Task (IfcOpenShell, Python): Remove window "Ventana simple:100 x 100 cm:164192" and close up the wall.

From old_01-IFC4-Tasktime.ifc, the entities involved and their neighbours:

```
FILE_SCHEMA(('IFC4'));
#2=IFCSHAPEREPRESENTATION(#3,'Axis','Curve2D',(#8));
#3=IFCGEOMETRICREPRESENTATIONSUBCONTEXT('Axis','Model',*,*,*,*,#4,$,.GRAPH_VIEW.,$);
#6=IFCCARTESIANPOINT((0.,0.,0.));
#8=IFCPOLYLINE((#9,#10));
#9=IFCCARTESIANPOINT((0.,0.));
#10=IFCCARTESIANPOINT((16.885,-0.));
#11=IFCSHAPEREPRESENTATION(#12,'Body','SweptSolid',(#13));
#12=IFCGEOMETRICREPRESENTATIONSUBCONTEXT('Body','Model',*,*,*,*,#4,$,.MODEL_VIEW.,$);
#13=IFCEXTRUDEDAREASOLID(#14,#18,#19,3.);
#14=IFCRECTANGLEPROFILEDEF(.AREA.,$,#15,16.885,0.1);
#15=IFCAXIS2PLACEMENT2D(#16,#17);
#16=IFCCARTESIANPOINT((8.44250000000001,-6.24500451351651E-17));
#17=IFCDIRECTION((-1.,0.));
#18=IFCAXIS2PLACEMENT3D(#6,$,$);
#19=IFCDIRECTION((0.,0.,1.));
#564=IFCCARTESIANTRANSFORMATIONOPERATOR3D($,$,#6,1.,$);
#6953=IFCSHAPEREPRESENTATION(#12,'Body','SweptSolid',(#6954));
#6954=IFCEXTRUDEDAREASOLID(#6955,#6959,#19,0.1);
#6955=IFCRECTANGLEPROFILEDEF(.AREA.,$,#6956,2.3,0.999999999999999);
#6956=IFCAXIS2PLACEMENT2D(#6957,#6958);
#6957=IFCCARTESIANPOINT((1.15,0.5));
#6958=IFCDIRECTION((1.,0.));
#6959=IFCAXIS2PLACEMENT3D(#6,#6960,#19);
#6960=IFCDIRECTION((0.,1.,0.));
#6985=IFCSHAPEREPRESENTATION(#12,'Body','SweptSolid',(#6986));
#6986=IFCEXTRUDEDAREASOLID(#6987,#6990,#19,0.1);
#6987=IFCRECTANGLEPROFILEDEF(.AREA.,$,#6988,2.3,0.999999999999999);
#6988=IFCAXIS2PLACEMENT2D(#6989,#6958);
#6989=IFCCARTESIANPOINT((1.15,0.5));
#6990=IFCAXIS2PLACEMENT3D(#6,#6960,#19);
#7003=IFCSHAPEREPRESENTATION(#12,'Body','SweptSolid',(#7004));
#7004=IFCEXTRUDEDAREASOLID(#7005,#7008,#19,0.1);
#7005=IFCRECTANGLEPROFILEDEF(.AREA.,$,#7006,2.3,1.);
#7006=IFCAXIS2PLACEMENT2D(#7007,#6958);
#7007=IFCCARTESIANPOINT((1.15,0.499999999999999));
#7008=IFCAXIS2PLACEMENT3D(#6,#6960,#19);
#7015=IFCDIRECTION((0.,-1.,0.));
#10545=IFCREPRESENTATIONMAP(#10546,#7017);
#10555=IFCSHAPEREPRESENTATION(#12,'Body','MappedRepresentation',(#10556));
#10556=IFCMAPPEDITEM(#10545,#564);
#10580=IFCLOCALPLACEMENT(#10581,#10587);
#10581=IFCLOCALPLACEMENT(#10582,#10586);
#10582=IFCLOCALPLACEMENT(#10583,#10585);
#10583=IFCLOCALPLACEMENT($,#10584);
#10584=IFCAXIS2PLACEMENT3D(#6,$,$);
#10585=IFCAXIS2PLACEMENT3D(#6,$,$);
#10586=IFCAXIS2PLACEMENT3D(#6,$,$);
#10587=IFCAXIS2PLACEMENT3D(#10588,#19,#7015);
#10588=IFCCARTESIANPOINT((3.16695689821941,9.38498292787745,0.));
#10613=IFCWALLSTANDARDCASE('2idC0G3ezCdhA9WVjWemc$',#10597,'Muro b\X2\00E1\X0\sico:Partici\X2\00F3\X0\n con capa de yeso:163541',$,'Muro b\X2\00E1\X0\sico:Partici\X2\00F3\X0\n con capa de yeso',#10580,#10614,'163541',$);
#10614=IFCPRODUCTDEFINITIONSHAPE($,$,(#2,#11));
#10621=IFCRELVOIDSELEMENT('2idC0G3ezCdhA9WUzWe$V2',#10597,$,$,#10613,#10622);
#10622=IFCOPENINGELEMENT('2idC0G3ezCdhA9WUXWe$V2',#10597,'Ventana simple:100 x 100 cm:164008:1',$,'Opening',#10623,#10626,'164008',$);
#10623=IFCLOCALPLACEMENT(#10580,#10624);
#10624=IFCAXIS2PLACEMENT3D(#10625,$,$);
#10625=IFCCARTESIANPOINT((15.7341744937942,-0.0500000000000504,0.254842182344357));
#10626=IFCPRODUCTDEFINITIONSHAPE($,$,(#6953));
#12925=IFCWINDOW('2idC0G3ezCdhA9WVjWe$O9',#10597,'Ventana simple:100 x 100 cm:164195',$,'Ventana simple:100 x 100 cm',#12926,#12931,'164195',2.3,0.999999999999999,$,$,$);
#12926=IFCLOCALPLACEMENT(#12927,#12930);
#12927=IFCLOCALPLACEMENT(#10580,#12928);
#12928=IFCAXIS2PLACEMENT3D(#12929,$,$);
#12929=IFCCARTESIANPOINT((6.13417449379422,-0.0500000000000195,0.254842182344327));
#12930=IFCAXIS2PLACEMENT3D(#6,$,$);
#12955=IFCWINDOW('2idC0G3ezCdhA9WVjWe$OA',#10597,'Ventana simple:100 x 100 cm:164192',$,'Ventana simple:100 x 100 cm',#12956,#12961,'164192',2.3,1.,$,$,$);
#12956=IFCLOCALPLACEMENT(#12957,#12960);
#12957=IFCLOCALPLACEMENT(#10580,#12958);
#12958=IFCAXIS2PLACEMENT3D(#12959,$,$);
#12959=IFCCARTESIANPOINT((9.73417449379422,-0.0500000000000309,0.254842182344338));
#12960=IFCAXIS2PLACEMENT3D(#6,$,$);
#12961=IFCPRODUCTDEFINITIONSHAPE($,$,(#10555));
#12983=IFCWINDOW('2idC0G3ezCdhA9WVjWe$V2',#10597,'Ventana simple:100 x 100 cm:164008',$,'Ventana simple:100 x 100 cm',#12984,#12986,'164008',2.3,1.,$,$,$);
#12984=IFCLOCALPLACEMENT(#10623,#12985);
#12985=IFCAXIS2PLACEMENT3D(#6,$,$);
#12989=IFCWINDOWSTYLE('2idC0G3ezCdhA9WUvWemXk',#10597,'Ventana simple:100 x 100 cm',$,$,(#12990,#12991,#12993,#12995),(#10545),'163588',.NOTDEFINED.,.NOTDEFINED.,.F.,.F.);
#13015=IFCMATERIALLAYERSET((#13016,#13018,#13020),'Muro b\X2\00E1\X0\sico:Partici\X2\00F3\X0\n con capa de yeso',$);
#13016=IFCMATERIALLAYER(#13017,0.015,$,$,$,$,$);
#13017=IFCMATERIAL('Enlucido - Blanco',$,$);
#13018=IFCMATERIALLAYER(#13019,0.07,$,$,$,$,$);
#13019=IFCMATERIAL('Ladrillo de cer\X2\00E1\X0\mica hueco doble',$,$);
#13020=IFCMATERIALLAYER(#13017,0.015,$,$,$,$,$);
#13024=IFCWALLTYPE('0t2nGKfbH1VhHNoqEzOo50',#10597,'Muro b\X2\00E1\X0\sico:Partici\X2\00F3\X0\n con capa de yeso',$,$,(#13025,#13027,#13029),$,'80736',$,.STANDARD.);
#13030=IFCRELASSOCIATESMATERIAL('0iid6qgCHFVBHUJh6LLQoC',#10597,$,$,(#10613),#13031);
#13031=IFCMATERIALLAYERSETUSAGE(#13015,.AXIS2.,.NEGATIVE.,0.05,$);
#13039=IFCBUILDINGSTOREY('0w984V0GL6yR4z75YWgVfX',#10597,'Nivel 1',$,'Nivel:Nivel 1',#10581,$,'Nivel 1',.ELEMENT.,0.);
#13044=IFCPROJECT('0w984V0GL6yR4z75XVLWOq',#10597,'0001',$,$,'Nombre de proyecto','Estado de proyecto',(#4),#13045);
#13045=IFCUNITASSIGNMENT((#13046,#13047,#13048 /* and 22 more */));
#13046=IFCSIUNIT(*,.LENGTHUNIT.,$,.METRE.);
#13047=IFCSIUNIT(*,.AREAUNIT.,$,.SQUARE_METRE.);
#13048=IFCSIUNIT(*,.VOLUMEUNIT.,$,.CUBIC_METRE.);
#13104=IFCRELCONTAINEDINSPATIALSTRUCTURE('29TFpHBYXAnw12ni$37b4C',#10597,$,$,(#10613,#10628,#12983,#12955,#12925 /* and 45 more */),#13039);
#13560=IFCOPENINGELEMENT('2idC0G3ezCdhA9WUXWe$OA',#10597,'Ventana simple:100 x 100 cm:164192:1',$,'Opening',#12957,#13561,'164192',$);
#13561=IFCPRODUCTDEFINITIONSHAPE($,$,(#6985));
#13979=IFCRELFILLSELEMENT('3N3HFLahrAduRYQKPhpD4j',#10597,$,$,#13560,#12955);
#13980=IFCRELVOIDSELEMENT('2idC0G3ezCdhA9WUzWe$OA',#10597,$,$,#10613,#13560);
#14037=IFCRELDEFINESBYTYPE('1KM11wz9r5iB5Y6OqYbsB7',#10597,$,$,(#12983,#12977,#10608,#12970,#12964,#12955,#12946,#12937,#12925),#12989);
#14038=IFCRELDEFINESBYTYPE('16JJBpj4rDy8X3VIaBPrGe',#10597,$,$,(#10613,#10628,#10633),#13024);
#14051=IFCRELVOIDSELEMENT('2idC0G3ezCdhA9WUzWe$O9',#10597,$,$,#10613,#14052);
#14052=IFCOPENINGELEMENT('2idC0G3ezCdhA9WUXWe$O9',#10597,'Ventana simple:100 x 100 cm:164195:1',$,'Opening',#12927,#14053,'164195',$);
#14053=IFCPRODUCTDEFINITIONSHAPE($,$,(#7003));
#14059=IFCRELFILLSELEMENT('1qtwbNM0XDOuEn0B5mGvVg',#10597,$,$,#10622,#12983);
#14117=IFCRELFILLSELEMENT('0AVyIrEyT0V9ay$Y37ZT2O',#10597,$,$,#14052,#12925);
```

```python
import ifcopenshell
import ifcopenshell.api.feature
import ifcopenshell.api.root
import ifcopenshell.geom
import ifcopenshell.util.shape

model = ifcopenshell.open("old_01-IFC4-Tasktime.ifc")
settings = ifcopenshell.geom.settings()


def volume(element):
    """Net volume in cubic metres, openings subtracted."""
    shape = ifcopenshell.geom.create_shape(settings, element)
    return ifcopenshell.util.shape.get_volume(shape.geometry)


window = model.by_guid("2idC0G3ezCdhA9WVjWe$OA")
opening = window.FillsVoids[0].RelatingOpeningElement
wall = opening.VoidsElements[0].RelatingBuildingElement
before = volume(wall)

ifcopenshell.api.root.remove_product(model, product=window)
ifcopenshell.api.feature.remove_feature(model, feature=opening)

after = volume(wall)

print(f"wall volume {before:.3f} -> {after:.3f} m3")

model.write("old_01-IFC4-Tasktime_v2.ifc")
```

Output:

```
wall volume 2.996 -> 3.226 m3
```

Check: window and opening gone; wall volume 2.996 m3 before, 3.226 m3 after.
